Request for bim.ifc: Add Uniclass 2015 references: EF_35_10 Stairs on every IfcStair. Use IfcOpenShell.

First a look at what the model holds.

```python
import ifcopenshell

model = ifcopenshell.open("bim.ifc")
print(model.schema)
print("classifications:", [c.Name for c in model.by_type("IfcClassification")])
for ifc_class in ("IfcDoor", "IfcRoof", "IfcStair", "IfcWall", "IfcWindow"):
    print(ifc_class, len(model.by_type(ifc_class)))
```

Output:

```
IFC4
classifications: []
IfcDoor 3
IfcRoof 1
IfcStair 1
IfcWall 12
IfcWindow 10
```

```python
import ifcopenshell
import ifcopenshell.api.classification

model = ifcopenshell.open("bim.ifc")

system = ifcopenshell.api.classification.add_classification(model, classification="Uniclass 2015")

codes = {
    "IfcStair": ("EF_35_10", "Stairs"),
}
for ifc_class, (code, name) in codes.items():
    products = model.by_type(ifc_class)
    ifcopenshell.api.classification.add_reference(
        model, products=products, classification=system, identification=code, name=name
    )
    print(code, len(products))

model.write("bim_edited.ifc")
```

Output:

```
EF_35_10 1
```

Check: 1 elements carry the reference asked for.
